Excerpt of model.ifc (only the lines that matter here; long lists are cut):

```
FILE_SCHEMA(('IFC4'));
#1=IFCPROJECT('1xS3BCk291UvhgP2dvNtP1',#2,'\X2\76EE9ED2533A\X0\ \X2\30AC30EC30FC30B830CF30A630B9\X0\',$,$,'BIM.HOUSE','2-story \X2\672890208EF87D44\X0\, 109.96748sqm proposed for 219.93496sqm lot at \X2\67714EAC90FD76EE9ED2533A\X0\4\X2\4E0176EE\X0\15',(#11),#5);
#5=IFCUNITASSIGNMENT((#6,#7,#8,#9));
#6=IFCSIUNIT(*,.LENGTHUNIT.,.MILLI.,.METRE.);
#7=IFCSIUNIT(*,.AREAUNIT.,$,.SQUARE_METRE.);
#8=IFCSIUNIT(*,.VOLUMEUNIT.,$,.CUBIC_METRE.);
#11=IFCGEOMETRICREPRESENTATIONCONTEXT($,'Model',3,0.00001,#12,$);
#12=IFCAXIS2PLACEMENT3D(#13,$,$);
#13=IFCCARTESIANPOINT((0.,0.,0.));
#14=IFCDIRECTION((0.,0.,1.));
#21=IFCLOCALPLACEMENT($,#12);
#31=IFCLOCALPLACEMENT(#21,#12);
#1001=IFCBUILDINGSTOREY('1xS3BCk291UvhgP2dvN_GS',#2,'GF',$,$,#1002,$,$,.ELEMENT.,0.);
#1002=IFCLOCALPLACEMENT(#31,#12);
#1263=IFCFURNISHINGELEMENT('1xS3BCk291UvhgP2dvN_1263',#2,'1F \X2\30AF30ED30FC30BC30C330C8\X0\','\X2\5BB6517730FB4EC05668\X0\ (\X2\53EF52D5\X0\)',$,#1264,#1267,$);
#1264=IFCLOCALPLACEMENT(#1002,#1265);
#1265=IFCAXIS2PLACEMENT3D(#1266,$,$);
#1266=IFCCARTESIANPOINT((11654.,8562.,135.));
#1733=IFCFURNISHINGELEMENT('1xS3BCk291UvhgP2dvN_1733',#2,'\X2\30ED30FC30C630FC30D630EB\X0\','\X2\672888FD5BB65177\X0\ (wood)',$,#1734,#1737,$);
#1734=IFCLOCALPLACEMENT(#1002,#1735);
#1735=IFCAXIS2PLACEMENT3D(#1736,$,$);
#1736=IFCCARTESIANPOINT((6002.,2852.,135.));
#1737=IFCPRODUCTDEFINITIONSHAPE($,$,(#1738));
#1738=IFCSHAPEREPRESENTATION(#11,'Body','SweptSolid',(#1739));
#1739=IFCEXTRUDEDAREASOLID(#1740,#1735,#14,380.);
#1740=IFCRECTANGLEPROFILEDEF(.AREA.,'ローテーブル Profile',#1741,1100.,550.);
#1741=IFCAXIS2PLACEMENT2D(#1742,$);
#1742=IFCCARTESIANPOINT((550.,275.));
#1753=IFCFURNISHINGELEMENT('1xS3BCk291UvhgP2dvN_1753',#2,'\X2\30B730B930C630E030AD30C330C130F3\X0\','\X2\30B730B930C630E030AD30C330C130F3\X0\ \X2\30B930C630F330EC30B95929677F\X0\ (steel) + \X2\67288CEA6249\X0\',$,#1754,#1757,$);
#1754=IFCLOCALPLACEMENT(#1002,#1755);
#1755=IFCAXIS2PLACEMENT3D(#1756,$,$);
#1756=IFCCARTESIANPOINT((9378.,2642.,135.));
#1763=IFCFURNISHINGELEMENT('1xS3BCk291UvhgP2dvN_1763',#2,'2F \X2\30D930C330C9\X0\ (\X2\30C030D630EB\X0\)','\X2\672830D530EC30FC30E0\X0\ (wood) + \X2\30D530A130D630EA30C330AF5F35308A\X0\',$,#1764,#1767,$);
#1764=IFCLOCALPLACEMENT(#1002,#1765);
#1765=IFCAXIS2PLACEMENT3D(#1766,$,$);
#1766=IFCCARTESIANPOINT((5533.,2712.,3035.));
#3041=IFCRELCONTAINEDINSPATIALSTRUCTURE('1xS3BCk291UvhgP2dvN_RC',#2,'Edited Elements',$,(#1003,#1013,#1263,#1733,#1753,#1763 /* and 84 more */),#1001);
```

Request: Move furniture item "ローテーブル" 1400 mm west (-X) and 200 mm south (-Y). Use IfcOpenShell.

```python
import ifcopenshell
import ifcopenshell.api.geometry
import ifcopenshell.util.placement
import ifcopenshell.util.unit

model = ifcopenshell.open("model.ifc")
unit_scale = ifcopenshell.util.unit.calculate_unit_scale(model)

item = model.by_guid("1xS3BCk291UvhgP2dvN_1733")
matrix = ifcopenshell.util.placement.get_local_placement(item.ObjectPlacement)
matrix[0, 3] -= 1.4 / unit_scale
matrix[1, 3] -= 0.2 / unit_scale
ifcopenshell.api.geometry.edit_object_placement(model, product=item, matrix=matrix, is_si=False)

print(ifcopenshell.util.placement.get_local_placement(item.ObjectPlacement).round(3) + 0.0)

model.write("model_v2.ifc")
```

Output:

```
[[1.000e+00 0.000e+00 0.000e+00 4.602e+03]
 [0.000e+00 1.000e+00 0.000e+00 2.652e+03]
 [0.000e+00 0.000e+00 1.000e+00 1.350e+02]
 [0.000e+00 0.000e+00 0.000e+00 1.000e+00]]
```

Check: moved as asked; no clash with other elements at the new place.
